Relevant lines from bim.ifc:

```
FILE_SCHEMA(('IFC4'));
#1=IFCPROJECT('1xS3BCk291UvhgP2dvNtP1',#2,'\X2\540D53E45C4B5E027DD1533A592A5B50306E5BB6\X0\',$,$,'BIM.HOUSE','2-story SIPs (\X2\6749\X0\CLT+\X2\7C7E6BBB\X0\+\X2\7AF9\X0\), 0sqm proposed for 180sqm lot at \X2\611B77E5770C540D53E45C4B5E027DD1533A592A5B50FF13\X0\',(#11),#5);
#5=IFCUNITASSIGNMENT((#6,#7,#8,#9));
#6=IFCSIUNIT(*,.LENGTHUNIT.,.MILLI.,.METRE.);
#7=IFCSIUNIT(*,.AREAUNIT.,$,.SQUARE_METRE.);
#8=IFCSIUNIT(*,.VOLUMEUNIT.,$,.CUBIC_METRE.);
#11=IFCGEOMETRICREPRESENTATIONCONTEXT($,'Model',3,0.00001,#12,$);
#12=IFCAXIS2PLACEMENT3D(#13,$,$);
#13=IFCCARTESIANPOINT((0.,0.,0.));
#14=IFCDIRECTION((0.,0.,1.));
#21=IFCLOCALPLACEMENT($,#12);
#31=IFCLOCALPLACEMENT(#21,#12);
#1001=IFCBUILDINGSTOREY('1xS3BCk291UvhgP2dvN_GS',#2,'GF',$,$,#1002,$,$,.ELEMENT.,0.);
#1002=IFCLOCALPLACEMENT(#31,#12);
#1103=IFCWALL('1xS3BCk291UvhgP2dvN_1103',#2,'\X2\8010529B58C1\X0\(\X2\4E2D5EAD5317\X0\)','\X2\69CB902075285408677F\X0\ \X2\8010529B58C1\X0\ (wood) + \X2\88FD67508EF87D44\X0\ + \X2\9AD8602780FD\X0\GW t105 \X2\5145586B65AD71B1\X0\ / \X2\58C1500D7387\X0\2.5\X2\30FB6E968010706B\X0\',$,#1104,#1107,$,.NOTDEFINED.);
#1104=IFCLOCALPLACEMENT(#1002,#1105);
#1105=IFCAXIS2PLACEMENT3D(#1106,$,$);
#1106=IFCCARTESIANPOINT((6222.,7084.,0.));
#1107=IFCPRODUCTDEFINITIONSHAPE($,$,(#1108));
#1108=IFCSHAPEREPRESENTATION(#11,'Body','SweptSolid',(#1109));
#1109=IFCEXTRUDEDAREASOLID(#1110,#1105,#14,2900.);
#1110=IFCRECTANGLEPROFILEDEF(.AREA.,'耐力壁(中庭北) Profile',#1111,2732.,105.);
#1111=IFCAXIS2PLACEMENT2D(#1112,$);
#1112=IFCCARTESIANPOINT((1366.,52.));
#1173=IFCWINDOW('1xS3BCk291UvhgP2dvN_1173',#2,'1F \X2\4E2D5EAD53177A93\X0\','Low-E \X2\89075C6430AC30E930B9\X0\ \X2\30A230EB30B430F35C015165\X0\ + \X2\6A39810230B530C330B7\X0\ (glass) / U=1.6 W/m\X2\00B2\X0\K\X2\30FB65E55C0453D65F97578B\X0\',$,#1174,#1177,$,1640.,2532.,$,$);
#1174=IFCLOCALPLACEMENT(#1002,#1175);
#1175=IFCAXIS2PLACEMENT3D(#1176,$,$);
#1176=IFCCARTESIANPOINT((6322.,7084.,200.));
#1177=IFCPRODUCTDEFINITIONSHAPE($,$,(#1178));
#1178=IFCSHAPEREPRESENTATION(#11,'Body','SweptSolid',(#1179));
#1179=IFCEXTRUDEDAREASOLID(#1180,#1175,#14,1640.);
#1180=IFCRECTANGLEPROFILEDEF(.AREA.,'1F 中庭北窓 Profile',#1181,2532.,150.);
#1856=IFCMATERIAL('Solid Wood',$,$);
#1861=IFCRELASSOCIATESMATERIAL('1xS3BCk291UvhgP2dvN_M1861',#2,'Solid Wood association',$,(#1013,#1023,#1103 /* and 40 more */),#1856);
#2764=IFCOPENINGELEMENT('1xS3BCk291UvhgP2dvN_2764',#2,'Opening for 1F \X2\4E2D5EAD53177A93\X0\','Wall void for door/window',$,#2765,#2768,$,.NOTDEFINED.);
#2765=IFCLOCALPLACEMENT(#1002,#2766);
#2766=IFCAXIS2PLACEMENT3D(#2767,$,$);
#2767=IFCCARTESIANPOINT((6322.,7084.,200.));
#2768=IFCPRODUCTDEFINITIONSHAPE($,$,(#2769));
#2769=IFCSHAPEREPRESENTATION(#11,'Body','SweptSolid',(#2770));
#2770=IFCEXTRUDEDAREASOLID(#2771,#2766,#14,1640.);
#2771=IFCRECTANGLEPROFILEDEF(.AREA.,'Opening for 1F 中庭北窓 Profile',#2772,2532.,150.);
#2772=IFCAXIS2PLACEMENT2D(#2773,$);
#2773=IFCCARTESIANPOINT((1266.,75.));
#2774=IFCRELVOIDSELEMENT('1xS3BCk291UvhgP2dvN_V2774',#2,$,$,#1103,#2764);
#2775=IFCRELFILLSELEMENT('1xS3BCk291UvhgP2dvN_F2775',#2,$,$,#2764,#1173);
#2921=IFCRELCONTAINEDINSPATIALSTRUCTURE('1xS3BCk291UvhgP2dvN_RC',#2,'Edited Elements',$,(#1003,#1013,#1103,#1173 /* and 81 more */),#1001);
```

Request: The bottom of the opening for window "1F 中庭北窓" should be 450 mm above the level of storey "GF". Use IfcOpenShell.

```python
import numpy as np
import ifcopenshell
import ifcopenshell.api.geometry
import ifcopenshell.geom
import ifcopenshell.util.element
import ifcopenshell.util.placement
import ifcopenshell.util.shape
import ifcopenshell.util.unit

model = ifcopenshell.open("bim.ifc")
unit_scale = ifcopenshell.util.unit.calculate_unit_scale(model)

window = model.by_guid("1xS3BCk291UvhgP2dvN_1173")
opening = window.FillsVoids[0].RelatingOpeningElement
storey = ifcopenshell.util.element.get_container(window, ifc_class="IfcBuildingStorey")
level = ifcopenshell.util.placement.get_local_placement(storey.ObjectPlacement)[2, 3]

# The opening's origin need not be at the sill, so measure its lowest point.
shape = ifcopenshell.geom.create_shape(ifcopenshell.geom.settings(), opening)
bottom = ifcopenshell.util.shape.get_shape_bottom_elevation(shape, shape.geometry) / unit_scale
dz = level + 450.0 - bottom

shift = np.array([0.0, 0.0, dz])
# The window is not placed relative to its opening, so move both.
for product in (opening, window):
    matrix = ifcopenshell.util.placement.get_local_placement(product.ObjectPlacement)
    matrix[:3, 3] += shift
    ifcopenshell.api.geometry.edit_object_placement(model, product=product, matrix=matrix, is_si=False)

print(f"moved by {dz * unit_scale:+.3f} m")

model.write("bim_edited.ifc")
```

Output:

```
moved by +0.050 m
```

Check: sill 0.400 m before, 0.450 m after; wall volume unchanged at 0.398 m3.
